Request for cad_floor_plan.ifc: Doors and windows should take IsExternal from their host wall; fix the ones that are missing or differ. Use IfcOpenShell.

First a look at what the model holds.

```python
import ifcopenshell
import ifcopenshell.util.element

model = ifcopenshell.open("cad_floor_plan.ifc")
print(model.schema)
seen = {}
for e in model.by_type("IfcDoor") + model.by_type("IfcWindow"):
    if not e.FillsVoids:
        continue
    host = e.FillsVoids[0].RelatingOpeningElement.VoidsElements[0].RelatingBuildingElement
    own = ifcopenshell.util.element.get_pset(e, f"Pset_{e.is_a()[3:].removesuffix('StandardCase')}Common", "IsExternal")
    wall = ifcopenshell.util.element.get_pset(host, "Pset_WallCommon", "IsExternal")
    seen[e.is_a(), own, wall] = seen.get((e.is_a(), own, wall), 0) + 1
for (cls, own, wall), count in sorted(seen.items(), key=str):
    print(count, cls, "IsExternal:", own, "| host wall:", wall)
```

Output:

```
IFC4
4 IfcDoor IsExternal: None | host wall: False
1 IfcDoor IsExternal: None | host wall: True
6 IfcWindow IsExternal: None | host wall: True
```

```python
import ifcopenshell
import ifcopenshell.api.pset
import ifcopenshell.util.element

model = ifcopenshell.open("cad_floor_plan.ifc")

count = 0
for ifc_class, pset_name in (("IfcDoor", "Pset_DoorCommon"), ("IfcWindow", "Pset_WindowCommon")):
    for e in model.by_type(ifc_class):
        if not e.FillsVoids:
            continue
        host = e.FillsVoids[0].RelatingOpeningElement.VoidsElements[0].RelatingBuildingElement
        external = ifcopenshell.util.element.get_pset(host, "Pset_WallCommon", "IsExternal")
        if external is None or ifcopenshell.util.element.get_pset(e, pset_name, "IsExternal") == external:
            continue
        pset = ifcopenshell.api.pset.add_pset(model, product=e, name=pset_name)
        ifcopenshell.api.pset.edit_pset(model, pset=pset, properties={"IsExternal": external})
        count += 1

print(count, "updated")

model.write("cad_floor_plan_rev.ifc")
```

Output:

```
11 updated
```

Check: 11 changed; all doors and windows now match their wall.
